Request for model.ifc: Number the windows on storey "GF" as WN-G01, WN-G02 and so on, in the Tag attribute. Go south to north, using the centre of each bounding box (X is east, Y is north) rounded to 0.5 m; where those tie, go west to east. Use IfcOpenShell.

First a look at what the model holds.

```python
import ifcopenshell
import ifcopenshell.util.element
import ifcopenshell.util.placement

model = ifcopenshell.open("model.ifc")
print(model.schema)
storey = next(s for s in model.by_type("IfcBuildingStorey") if s.Name == "GF")
windows = [e for e in ifcopenshell.util.element.get_decomposition(storey) if e.is_a("IfcWindow")]
for e in sorted(windows, key=lambda e: e.id()):
    origin = ifcopenshell.util.placement.get_local_placement(e.ObjectPlacement)[:3, 3]
    print(e.id(), e.Tag, e.Name, origin.round(2) + 0.0, sep=" | ")
```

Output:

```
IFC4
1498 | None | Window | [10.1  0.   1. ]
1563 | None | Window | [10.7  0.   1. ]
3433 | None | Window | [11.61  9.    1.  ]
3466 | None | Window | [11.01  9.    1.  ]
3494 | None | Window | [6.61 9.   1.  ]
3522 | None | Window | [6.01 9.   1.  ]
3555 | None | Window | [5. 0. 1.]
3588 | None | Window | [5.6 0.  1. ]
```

```python
import ifcopenshell
import ifcopenshell.geom
import ifcopenshell.util.element
import ifcopenshell.util.shape

model = ifcopenshell.open("model.ifc")
settings = ifcopenshell.geom.settings()
settings.set("use-world-coords", True)


def centre(element):
    shape = ifcopenshell.geom.create_shape(settings, element)
    return ifcopenshell.util.shape.get_bbox_centroid(shape.geometry)


storey = next(s for s in model.by_type("IfcBuildingStorey") if s.Name == "GF")
windows = [e for e in ifcopenshell.util.element.get_decomposition(storey) if e.is_a("IfcWindow")]

# Insertion points can sit at a corner or the storey origin, so sort by the geometry (in metres).
centres = {e: centre(e) for e in windows}
windows.sort(key=lambda e: (round(centres[e][1] / 0.5), centres[e][0]))

for i, e in enumerate(windows, start=1):
    number = f"WN-G{i:02d}"
    e.Tag = number
    print(e.id(), number)

model.write("model_edited.ifc")
```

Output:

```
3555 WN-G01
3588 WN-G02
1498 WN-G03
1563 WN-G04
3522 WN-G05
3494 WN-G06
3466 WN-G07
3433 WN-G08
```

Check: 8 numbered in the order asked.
